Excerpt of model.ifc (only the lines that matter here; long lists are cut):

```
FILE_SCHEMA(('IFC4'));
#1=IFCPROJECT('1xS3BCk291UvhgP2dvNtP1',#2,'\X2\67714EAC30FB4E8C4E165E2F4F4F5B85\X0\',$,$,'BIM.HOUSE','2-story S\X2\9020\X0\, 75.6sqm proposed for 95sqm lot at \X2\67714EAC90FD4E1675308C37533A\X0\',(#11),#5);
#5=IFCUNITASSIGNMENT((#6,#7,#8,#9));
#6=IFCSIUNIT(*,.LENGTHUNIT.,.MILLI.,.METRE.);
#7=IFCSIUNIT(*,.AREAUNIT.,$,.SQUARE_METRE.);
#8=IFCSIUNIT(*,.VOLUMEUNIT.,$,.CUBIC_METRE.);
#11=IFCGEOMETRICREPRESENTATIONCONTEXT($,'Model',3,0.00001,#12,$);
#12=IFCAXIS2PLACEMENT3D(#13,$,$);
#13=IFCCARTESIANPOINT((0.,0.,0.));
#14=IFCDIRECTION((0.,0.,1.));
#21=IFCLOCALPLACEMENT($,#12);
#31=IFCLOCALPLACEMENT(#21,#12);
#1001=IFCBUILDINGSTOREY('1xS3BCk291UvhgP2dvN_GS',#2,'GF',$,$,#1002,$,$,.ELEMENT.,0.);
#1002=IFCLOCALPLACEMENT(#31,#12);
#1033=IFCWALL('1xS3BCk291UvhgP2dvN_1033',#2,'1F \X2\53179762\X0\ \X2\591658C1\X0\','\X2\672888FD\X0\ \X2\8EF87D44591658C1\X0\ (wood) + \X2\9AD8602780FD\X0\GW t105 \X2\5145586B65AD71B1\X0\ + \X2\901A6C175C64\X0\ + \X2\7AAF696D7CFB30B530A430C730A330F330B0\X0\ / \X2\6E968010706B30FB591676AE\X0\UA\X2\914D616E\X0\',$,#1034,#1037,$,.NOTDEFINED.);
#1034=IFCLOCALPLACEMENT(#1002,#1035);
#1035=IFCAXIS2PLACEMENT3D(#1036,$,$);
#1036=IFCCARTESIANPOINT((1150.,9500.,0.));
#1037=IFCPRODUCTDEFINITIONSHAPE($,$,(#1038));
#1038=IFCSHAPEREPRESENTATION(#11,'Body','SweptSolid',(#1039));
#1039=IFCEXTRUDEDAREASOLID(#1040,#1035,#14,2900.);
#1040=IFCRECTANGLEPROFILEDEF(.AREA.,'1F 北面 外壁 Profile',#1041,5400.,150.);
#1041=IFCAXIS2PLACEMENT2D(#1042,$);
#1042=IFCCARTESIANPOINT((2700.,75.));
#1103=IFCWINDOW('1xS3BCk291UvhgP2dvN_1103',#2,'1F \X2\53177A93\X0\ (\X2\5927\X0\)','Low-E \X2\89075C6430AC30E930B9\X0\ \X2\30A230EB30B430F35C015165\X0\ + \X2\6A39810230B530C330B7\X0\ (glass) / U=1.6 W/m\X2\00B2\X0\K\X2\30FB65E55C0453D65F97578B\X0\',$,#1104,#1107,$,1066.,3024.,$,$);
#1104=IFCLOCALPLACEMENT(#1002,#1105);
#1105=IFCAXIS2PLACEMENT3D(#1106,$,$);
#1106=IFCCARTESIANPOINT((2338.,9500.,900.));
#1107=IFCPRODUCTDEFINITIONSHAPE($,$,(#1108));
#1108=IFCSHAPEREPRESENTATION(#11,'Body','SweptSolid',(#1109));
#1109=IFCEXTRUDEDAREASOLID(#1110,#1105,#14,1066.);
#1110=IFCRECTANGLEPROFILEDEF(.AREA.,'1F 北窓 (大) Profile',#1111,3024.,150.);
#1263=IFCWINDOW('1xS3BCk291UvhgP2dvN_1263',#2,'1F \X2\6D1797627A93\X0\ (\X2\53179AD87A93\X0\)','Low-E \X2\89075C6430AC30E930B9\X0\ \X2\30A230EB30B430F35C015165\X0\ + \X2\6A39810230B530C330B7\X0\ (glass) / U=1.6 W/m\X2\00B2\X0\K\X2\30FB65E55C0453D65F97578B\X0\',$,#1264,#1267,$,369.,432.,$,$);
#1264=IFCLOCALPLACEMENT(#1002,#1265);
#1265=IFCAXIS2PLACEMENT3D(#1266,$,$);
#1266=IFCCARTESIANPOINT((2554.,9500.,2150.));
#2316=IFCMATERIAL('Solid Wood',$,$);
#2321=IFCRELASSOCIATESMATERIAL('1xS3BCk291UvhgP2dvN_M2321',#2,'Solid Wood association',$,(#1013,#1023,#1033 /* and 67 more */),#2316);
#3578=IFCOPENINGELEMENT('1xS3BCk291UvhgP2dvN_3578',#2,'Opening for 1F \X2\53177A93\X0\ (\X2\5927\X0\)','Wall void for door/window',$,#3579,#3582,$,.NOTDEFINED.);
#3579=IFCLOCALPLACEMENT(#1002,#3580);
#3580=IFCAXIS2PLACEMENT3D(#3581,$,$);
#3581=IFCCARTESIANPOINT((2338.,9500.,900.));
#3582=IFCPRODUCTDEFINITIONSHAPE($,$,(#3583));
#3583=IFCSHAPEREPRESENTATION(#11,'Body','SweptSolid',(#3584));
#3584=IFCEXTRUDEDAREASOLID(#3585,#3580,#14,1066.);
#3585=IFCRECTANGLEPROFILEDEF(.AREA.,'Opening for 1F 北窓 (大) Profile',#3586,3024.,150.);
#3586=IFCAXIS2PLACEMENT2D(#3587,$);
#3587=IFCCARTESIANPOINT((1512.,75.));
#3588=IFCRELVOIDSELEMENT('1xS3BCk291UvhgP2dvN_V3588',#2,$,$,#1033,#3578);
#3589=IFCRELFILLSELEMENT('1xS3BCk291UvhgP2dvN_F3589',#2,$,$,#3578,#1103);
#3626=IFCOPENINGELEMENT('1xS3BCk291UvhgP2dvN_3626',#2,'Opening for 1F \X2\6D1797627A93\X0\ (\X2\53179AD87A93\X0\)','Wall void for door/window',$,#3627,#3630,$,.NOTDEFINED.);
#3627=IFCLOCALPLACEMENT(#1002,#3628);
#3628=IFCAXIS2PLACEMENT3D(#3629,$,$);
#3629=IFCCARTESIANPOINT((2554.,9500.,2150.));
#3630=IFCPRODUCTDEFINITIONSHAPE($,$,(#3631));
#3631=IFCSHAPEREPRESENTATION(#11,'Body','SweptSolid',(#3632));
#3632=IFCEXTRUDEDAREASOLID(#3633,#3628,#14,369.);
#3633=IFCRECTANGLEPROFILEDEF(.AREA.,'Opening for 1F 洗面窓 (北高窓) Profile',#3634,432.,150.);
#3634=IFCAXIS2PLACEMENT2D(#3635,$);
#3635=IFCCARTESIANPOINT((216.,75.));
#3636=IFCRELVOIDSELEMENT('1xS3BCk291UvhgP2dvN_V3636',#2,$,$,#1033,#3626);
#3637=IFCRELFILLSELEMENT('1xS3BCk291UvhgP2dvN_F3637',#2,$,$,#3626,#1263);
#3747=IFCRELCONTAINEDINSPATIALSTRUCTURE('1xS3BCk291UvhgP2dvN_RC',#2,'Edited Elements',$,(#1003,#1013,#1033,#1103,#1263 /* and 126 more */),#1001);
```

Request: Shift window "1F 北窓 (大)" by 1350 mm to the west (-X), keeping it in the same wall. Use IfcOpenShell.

```python
import ifcopenshell
import ifcopenshell.api.geometry
import ifcopenshell.util.placement
import ifcopenshell.util.unit

model = ifcopenshell.open("model.ifc")
unit_scale = ifcopenshell.util.unit.calculate_unit_scale(model)

window = model.by_guid("1xS3BCk291UvhgP2dvN_1103")
opening = window.FillsVoids[0].RelatingOpeningElement
wall = opening.VoidsElements[0].RelatingBuildingElement

wall_matrix = ifcopenshell.util.placement.get_local_placement(wall.ObjectPlacement)
shift = wall_matrix[:3, 0] * -1.35 / unit_scale
before = ifcopenshell.util.placement.get_local_placement(window.ObjectPlacement)[:3, 3].copy()

# The window is not placed relative to its opening, so move both.
for product in (opening, window):
    matrix = ifcopenshell.util.placement.get_local_placement(product.ObjectPlacement)
    matrix[:3, 3] += shift
    ifcopenshell.api.geometry.edit_object_placement(model, product=product, matrix=matrix, is_si=False)

after = ifcopenshell.util.placement.get_local_placement(window.ObjectPlacement)[:3, 3]
print("window moved by", (after - before).round(3) + 0.0)

model.write("model-out.ifc")
```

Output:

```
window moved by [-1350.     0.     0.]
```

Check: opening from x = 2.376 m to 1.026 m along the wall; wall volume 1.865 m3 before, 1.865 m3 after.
